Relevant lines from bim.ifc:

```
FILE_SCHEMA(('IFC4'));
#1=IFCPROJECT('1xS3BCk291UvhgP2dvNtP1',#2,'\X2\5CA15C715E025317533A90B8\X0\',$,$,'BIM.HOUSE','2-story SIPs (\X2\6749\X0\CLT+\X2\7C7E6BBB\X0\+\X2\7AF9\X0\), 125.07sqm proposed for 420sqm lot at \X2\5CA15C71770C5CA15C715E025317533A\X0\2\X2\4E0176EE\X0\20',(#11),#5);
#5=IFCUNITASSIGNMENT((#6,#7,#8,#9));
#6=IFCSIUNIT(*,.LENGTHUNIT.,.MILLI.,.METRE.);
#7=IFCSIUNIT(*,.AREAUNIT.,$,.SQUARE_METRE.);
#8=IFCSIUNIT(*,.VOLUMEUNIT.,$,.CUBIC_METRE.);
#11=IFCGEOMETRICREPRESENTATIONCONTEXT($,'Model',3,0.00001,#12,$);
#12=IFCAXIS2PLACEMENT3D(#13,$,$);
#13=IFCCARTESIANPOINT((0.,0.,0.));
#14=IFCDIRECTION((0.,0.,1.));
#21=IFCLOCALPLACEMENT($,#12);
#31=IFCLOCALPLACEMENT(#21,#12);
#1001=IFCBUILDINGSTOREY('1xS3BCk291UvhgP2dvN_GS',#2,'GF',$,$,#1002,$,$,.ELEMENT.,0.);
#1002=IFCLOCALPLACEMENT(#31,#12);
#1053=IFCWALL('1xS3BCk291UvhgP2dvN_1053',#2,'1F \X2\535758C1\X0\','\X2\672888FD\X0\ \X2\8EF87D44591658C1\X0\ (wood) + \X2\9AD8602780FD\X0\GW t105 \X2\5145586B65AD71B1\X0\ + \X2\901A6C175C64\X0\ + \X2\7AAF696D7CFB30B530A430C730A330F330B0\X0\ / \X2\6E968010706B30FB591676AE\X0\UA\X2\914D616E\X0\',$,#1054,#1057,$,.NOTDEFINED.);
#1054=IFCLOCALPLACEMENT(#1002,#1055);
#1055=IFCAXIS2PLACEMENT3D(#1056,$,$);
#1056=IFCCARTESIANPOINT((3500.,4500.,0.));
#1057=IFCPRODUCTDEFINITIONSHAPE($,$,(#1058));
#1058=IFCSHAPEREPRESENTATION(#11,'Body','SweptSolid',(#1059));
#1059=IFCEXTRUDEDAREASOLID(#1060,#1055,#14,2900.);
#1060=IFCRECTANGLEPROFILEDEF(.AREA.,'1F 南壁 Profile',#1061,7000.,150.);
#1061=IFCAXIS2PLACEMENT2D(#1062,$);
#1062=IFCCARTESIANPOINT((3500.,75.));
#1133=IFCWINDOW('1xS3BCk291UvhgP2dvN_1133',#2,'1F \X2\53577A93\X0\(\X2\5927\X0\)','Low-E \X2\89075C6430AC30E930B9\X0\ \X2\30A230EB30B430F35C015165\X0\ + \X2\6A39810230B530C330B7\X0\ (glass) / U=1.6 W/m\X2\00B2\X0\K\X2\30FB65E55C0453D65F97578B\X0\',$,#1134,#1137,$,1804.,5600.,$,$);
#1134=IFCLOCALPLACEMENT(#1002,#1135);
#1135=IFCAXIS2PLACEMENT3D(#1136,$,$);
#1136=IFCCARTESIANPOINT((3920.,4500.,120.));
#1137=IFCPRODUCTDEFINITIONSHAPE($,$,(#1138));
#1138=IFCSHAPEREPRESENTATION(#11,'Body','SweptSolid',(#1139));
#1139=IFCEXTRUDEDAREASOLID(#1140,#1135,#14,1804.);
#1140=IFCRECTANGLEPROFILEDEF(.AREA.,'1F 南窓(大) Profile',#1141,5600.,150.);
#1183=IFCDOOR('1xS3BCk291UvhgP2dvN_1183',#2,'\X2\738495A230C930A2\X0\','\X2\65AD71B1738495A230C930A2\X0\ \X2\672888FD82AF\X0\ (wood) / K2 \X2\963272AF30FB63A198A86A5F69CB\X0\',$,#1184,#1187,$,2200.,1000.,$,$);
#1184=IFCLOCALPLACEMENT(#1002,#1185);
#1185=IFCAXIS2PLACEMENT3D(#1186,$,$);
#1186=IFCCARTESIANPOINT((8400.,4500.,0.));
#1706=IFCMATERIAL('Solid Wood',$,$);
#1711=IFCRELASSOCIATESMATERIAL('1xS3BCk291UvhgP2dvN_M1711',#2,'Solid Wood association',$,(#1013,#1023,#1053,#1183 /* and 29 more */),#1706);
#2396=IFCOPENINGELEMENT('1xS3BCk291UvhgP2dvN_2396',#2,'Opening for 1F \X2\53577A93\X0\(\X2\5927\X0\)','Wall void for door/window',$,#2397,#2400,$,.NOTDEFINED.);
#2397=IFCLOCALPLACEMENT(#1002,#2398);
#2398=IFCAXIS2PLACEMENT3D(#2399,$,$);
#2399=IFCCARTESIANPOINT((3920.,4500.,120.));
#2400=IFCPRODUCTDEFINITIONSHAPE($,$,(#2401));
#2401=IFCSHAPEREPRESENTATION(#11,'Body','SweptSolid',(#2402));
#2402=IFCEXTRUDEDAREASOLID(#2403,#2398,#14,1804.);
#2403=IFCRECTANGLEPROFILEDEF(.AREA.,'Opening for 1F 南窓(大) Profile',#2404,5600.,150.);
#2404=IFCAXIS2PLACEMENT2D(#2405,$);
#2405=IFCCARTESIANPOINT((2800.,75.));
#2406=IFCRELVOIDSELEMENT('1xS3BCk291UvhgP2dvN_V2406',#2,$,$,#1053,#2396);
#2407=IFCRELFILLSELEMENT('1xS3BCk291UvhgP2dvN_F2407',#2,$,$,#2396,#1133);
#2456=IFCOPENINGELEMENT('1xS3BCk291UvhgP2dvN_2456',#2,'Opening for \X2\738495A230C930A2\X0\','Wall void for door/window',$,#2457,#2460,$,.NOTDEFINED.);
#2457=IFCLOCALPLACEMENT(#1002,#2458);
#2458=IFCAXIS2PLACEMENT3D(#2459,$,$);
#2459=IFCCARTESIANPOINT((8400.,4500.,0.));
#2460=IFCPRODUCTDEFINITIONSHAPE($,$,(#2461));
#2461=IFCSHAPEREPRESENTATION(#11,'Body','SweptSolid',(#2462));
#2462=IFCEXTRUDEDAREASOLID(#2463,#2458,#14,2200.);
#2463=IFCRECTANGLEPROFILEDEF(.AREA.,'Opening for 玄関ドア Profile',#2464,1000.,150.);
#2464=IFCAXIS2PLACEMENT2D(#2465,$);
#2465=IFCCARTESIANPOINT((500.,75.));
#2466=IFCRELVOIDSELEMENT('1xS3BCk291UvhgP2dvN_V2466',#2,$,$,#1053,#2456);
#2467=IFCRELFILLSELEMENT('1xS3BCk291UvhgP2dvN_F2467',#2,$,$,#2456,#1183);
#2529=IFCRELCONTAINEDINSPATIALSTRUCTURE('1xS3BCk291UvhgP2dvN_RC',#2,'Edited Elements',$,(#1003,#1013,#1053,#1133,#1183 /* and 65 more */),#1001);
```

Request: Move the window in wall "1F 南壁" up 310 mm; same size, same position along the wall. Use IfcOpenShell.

```python
import numpy as np
import ifcopenshell
import ifcopenshell.api.geometry
import ifcopenshell.util.placement
import ifcopenshell.util.unit

model = ifcopenshell.open("bim.ifc")
unit_scale = ifcopenshell.util.unit.calculate_unit_scale(model)

window = model.by_guid("1xS3BCk291UvhgP2dvN_1133")
opening = window.FillsVoids[0].RelatingOpeningElement
dz = 0.31 / unit_scale

shift = np.array([0.0, 0.0, dz])
# The window is not placed relative to its opening, so move both.
for product in (opening, window):
    matrix = ifcopenshell.util.placement.get_local_placement(product.ObjectPlacement)
    matrix[:3, 3] += shift
    ifcopenshell.api.geometry.edit_object_placement(model, product=product, matrix=matrix, is_si=False)

print(f"moved by {dz * unit_scale:+.3f} m")

model.write("bim-out.ifc")
```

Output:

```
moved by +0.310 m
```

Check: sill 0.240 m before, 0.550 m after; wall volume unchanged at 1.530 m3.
